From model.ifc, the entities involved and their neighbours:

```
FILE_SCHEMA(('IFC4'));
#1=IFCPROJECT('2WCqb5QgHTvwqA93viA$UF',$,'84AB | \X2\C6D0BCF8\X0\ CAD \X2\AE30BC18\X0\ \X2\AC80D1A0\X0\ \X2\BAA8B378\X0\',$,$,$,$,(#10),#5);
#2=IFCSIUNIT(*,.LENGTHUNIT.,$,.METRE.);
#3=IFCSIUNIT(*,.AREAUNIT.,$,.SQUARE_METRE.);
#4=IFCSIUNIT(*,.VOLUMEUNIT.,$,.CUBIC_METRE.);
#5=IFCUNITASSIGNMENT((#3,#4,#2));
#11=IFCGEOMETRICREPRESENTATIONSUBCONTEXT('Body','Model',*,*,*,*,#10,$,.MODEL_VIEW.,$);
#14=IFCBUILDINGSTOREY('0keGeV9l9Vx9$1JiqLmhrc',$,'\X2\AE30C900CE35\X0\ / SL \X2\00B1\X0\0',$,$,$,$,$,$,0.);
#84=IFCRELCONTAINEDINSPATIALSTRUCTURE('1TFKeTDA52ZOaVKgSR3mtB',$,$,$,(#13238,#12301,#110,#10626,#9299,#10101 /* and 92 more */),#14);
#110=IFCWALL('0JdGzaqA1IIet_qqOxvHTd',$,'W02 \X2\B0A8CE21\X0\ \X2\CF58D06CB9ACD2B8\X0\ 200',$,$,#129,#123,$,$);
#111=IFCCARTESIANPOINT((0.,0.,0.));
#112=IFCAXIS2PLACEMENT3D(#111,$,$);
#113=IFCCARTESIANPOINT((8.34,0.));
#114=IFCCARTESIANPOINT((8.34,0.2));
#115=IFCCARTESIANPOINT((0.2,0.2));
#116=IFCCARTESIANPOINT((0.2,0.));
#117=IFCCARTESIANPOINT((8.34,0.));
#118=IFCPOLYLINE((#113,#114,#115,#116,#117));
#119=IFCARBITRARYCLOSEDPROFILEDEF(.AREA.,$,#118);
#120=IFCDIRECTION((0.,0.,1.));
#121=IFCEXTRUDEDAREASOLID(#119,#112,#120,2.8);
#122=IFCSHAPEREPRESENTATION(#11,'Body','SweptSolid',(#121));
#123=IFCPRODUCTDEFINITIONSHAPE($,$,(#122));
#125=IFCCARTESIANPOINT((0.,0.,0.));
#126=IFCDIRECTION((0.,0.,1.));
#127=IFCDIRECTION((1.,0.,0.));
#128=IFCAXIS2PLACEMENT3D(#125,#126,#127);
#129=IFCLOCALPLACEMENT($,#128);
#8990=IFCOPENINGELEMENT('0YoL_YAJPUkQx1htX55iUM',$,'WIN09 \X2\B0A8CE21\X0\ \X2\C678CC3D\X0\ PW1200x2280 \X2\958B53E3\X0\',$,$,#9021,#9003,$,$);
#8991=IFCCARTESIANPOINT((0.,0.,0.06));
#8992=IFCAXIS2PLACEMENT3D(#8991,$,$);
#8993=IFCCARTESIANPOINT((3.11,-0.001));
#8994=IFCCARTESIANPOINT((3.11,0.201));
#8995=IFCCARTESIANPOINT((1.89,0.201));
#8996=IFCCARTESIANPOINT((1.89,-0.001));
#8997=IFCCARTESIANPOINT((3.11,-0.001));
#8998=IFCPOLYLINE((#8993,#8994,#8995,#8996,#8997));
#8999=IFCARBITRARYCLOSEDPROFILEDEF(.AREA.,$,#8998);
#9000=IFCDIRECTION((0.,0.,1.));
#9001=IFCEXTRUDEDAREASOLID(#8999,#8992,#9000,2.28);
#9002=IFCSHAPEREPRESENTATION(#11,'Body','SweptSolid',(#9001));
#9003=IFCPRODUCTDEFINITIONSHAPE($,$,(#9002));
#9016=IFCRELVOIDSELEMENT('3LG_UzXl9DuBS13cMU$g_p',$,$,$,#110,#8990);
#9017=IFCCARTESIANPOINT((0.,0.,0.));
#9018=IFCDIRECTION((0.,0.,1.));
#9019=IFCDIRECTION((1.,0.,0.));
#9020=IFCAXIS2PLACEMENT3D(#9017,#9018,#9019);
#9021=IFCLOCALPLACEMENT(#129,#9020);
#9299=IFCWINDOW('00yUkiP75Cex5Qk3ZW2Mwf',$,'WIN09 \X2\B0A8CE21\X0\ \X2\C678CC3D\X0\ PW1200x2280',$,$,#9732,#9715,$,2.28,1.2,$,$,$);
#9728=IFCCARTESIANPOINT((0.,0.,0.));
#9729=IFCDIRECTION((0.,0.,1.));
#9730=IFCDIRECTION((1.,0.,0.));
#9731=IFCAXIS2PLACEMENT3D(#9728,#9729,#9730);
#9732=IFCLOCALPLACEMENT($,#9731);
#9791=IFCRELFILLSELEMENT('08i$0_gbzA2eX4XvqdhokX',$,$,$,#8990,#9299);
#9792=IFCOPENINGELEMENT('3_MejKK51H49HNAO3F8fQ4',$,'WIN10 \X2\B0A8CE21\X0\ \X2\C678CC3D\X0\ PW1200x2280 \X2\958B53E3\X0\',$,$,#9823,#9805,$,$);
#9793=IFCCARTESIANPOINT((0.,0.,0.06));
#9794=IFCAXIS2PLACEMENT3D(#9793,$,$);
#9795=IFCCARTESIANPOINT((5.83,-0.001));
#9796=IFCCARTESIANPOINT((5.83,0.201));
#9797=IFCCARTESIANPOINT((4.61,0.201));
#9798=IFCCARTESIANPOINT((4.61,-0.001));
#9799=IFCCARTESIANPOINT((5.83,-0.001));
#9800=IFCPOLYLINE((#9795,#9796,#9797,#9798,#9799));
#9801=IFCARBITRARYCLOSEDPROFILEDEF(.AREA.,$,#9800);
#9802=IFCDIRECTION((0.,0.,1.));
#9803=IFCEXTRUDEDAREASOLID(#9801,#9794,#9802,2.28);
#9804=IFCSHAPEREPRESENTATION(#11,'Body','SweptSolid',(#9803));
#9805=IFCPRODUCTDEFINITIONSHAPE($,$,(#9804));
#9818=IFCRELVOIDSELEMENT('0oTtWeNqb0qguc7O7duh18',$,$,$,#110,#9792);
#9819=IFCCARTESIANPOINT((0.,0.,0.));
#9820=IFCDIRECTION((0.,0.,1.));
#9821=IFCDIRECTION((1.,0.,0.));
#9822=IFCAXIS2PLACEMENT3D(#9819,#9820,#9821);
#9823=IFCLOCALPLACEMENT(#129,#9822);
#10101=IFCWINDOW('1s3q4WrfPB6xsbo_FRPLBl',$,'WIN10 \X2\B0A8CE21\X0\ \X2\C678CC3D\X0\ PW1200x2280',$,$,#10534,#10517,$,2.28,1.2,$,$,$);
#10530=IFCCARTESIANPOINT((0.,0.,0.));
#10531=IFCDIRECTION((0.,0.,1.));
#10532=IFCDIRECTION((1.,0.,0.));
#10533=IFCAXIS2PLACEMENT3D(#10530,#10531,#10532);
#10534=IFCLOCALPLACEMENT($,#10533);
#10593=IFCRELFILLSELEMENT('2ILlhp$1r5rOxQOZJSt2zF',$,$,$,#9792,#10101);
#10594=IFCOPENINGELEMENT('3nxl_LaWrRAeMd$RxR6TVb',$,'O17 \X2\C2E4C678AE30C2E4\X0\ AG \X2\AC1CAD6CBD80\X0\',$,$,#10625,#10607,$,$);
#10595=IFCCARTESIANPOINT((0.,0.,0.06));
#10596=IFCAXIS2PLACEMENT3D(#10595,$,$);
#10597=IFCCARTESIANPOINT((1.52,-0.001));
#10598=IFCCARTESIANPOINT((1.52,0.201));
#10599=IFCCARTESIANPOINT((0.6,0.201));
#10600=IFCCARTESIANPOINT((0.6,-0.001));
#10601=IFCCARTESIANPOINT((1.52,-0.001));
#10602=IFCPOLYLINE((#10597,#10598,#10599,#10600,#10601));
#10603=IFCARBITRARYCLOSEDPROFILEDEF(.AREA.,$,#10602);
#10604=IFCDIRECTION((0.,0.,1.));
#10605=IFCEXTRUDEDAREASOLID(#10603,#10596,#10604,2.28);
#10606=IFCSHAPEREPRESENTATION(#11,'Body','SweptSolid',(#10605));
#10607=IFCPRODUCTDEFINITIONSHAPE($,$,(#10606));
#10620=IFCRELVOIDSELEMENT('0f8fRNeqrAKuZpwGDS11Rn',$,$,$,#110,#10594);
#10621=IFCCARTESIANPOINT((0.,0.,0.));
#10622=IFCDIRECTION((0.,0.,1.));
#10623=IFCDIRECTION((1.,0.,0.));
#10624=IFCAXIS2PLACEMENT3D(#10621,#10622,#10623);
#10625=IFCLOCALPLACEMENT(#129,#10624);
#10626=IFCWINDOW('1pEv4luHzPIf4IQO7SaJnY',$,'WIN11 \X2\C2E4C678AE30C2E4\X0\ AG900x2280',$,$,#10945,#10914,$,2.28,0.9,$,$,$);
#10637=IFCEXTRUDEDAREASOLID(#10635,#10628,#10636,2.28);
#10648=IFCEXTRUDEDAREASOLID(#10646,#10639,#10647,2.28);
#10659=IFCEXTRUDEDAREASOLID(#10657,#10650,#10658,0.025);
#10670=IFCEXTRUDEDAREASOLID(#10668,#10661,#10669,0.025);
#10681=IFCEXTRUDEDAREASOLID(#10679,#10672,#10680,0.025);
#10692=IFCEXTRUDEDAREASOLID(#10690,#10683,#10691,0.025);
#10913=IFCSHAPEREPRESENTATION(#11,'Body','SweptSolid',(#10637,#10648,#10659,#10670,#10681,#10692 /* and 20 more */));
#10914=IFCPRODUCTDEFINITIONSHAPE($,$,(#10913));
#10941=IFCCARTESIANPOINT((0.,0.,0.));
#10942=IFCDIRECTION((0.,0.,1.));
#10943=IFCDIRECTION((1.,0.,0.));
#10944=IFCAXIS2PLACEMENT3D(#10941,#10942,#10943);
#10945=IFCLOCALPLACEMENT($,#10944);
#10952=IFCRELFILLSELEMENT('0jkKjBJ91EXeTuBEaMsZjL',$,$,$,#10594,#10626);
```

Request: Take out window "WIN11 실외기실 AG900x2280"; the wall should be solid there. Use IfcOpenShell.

```python
import ifcopenshell
import ifcopenshell.api.feature
import ifcopenshell.api.root
import ifcopenshell.geom
import ifcopenshell.util.shape

model = ifcopenshell.open("model.ifc")
settings = ifcopenshell.geom.settings()


def volume(element):
    """Net volume in cubic metres, openings subtracted."""
    shape = ifcopenshell.geom.create_shape(settings, element)
    return ifcopenshell.util.shape.get_volume(shape.geometry)


window = model.by_guid("1pEv4luHzPIf4IQO7SaJnY")
opening = window.FillsVoids[0].RelatingOpeningElement
wall = opening.VoidsElements[0].RelatingBuildingElement
before = volume(wall)

ifcopenshell.api.root.remove_product(model, product=window)
ifcopenshell.api.feature.remove_feature(model, feature=opening)

after = volume(wall)

print(f"wall volume {before:.3f} -> {after:.3f} m3")

model.write("model_rev.ifc")
```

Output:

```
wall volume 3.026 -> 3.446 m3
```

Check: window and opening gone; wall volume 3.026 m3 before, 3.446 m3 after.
